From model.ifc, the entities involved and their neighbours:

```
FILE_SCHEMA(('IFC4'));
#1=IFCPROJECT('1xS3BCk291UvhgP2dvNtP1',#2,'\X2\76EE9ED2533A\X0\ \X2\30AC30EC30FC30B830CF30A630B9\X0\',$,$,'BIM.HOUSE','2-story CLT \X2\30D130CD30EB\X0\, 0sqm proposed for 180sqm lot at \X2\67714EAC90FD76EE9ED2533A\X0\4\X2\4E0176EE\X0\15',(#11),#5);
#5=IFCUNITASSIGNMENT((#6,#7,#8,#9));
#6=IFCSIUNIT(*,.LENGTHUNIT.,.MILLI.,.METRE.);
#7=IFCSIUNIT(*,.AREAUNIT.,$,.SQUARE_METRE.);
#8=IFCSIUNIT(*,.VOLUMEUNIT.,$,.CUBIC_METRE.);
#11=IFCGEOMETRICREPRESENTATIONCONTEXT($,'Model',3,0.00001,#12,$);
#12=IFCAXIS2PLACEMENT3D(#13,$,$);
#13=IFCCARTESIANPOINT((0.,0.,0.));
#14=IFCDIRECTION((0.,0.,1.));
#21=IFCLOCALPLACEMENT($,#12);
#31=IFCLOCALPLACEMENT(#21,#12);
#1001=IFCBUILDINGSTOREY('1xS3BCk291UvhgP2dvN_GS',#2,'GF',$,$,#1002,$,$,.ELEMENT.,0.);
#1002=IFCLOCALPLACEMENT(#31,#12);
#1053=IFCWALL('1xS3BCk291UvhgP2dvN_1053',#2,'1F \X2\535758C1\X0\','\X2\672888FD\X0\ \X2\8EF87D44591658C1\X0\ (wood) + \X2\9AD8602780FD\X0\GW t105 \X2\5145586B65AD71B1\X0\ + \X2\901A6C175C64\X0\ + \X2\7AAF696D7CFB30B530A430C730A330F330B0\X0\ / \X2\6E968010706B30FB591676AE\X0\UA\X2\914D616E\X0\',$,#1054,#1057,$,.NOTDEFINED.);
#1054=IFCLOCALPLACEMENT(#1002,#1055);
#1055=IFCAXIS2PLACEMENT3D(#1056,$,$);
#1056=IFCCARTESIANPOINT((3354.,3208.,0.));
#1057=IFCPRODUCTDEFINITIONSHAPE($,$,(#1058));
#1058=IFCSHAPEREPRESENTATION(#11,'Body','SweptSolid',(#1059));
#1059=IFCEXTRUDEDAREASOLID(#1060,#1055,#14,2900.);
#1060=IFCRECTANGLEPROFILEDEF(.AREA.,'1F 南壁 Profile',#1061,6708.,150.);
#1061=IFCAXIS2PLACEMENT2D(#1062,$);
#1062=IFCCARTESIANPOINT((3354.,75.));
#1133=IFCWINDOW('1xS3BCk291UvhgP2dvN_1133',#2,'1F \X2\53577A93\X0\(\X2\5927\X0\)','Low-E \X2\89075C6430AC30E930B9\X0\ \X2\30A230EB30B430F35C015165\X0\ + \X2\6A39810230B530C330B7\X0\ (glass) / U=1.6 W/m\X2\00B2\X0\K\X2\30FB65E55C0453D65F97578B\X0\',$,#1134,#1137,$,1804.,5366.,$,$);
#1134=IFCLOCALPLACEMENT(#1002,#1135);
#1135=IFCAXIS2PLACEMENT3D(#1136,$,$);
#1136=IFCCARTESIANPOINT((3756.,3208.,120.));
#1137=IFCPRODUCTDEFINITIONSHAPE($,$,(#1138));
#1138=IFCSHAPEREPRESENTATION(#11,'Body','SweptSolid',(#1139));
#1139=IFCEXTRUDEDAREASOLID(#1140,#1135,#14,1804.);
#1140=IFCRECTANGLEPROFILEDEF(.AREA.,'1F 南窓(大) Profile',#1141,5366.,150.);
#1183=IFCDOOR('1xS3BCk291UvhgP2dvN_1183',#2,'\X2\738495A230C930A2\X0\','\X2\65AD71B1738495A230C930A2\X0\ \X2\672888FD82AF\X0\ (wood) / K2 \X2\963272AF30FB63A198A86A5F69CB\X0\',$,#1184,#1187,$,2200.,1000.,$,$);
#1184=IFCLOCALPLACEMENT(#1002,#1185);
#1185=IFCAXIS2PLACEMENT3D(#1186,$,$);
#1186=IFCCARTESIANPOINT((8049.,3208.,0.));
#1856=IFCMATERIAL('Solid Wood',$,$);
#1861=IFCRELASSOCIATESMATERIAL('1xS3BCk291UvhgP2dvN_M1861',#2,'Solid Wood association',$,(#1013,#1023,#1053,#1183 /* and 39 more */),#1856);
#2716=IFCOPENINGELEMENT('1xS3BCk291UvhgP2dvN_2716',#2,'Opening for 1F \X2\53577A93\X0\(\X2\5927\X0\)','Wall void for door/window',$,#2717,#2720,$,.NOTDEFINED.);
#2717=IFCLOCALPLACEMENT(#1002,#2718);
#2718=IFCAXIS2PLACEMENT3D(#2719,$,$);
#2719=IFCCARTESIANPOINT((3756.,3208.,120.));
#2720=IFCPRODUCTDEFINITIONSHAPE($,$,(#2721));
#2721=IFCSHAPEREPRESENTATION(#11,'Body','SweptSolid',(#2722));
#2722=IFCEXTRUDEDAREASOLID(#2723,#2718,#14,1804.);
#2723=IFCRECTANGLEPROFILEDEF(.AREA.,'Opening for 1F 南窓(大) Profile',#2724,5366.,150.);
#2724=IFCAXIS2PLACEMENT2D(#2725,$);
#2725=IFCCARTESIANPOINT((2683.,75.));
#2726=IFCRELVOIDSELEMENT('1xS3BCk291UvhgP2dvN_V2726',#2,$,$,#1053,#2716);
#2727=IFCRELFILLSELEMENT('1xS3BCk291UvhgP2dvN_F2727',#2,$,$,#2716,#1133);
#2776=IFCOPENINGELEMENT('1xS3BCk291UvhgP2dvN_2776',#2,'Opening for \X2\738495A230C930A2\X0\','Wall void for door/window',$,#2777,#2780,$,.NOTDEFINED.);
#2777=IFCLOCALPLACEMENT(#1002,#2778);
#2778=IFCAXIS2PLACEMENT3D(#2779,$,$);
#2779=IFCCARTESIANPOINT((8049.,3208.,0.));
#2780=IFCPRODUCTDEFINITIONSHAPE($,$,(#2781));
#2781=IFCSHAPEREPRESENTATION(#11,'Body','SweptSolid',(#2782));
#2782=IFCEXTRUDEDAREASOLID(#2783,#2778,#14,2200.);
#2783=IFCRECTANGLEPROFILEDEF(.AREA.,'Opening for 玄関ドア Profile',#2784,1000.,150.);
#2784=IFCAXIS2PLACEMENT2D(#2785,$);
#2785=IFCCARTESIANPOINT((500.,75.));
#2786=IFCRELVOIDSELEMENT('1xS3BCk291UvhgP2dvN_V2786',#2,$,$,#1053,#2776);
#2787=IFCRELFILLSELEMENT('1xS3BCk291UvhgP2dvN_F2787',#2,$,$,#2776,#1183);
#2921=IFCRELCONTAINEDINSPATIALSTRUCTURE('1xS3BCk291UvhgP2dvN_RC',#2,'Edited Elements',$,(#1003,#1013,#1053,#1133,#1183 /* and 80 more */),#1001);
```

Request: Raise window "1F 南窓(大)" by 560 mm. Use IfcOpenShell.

```python
import numpy as np
import ifcopenshell
import ifcopenshell.api.geometry
import ifcopenshell.util.placement
import ifcopenshell.util.unit

model = ifcopenshell.open("model.ifc")
unit_scale = ifcopenshell.util.unit.calculate_unit_scale(model)

window = model.by_guid("1xS3BCk291UvhgP2dvN_1133")
opening = window.FillsVoids[0].RelatingOpeningElement
dz = 0.56 / unit_scale

shift = np.array([0.0, 0.0, dz])
# The window is not placed relative to its opening, so move both.
for product in (opening, window):
    matrix = ifcopenshell.util.placement.get_local_placement(product.ObjectPlacement)
    matrix[:3, 3] += shift
    ifcopenshell.api.geometry.edit_object_placement(model, product=product, matrix=matrix, is_si=False)

print(f"moved by {dz * unit_scale:+.3f} m")

model.write("model-out.ifc")
```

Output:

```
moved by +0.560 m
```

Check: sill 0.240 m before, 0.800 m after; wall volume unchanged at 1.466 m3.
